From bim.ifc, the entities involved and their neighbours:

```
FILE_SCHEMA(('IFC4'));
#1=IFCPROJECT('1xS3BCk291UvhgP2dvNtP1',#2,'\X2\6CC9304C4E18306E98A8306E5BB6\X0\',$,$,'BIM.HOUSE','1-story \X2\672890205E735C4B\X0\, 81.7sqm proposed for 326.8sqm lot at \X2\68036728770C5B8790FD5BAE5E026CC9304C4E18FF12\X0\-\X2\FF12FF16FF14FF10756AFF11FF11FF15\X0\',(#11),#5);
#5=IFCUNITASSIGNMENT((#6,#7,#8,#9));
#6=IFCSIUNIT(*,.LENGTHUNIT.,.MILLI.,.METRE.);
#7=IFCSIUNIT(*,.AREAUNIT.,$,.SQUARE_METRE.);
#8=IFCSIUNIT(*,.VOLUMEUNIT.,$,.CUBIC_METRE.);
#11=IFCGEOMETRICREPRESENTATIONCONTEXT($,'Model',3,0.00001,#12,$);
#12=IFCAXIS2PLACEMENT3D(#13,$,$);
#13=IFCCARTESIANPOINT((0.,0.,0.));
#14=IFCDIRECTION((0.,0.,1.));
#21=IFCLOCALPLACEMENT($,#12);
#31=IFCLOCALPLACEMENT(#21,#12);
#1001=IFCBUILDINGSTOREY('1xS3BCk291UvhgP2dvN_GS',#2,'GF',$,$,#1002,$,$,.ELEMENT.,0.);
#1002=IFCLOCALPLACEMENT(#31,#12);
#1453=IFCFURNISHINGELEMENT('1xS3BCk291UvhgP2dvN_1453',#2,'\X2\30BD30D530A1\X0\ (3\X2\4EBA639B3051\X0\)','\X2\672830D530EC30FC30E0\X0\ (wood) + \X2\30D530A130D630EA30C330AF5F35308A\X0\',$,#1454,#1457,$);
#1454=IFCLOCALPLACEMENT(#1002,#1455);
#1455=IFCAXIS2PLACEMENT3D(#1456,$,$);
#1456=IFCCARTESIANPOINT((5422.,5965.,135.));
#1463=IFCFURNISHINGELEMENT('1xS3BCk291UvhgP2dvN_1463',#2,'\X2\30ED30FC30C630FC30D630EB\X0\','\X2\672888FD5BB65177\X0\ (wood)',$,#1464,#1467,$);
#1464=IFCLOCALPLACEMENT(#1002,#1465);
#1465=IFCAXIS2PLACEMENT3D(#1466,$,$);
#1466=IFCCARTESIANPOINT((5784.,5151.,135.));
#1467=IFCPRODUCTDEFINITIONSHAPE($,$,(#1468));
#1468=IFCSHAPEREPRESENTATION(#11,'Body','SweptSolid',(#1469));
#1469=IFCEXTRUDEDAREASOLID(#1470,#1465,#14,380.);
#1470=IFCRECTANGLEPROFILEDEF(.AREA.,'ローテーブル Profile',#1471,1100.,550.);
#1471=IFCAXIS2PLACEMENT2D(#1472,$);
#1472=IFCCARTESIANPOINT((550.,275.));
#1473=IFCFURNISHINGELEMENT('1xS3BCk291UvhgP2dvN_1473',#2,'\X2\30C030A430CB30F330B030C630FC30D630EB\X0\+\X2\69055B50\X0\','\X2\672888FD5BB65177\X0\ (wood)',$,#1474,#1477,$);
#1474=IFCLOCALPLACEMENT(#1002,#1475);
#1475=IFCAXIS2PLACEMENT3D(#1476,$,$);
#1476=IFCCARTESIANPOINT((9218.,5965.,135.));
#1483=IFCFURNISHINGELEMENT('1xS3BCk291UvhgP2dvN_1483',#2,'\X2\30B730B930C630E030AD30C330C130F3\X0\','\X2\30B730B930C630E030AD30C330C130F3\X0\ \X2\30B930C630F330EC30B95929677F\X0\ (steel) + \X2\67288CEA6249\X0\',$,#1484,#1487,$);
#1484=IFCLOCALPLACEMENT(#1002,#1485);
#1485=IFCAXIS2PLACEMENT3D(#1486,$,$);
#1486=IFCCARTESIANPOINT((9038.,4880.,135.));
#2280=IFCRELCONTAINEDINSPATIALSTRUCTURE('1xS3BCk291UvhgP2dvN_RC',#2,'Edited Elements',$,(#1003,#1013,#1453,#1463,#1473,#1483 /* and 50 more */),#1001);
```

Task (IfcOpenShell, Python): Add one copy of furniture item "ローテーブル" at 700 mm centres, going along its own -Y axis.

```python
import ifcopenshell
import ifcopenshell.api.geometry
import ifcopenshell.api.root
import ifcopenshell.util.element
import ifcopenshell.util.placement
import ifcopenshell.util.unit

model = ifcopenshell.open("bim.ifc")
unit_scale = ifcopenshell.util.unit.calculate_unit_scale(model)


def reuse_history(source, copy):
    """copy_class also copies each property set's owner history, people and application; keep the originals."""
    for rel in copy.IsDefinedBy:
        if rel.is_a("IfcRelDefinesByProperties") and (history := rel.RelatingPropertyDefinition.OwnerHistory):
            rel.RelatingPropertyDefinition.OwnerHistory = source.OwnerHistory
            ifcopenshell.util.element.remove_deep2(model, history)


source = model.by_guid("1xS3BCk291UvhgP2dvN_1463")
base = ifcopenshell.util.placement.get_local_placement(source.ObjectPlacement)
step = -base[:3, 1] * 0.7 / unit_scale

for i in range(1, 2):
    copy = ifcopenshell.api.root.copy_class(model, product=source)
    copy.Representation = ifcopenshell.util.element.copy_deep(
        model, source.Representation, exclude=["IfcGeometricRepresentationContext", "IfcRepresentationMap"]
    )
    reuse_history(source, copy)
    matrix = base.copy()
    matrix[:3, 3] += i * step
    print("added at", matrix[:3, 3].round(3) + 0.0)
    ifcopenshell.api.geometry.edit_object_placement(model, product=copy, matrix=matrix, is_si=False)

model.write("bim_v2.ifc")
```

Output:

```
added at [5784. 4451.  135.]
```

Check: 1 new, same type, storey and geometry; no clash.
